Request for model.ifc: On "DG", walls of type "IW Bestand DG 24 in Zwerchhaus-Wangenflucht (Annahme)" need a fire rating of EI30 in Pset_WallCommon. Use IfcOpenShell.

First a look at what the model holds.

```python
import ifcopenshell
import ifcopenshell.util.element

model = ifcopenshell.open("model.ifc")
print(model.schema)
storey = next(s for s in model.by_type("IfcBuildingStorey") if s.Name == "DG")
walls = [e for e in ifcopenshell.util.element.get_decomposition(storey) if e.is_a("IfcWall")]
seen = {}
for e in walls:
    element_type = ifcopenshell.util.element.get_type(e)
    key = (element_type.Name if element_type != e and element_type else None, ifcopenshell.util.element.get_pset(e, "Pset_WallCommon", "FireRating"))
    seen[key] = seen.get(key, 0) + 1
for (name, value), count in sorted(seen.items(), key=str):
    print(count, "x", name, "|", value)
```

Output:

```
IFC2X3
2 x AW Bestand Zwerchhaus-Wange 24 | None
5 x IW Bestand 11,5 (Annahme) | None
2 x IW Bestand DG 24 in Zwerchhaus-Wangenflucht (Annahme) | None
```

```python
import ifcopenshell
import ifcopenshell.api.pset
import ifcopenshell.util.element

model = ifcopenshell.open("model.ifc")

storey = next(s for s in model.by_type("IfcBuildingStorey") if s.Name == "DG")
walls = [e for e in ifcopenshell.util.element.get_decomposition(storey) if e.is_a("IfcWall")]

count = 0
for e in walls:
    element_type = ifcopenshell.util.element.get_type(e)
    if element_type in (None, e) or element_type.Name != "IW Bestand DG 24 in Zwerchhaus-Wangenflucht (Annahme)":
        continue
    # add_pset returns the element's existing set when there is one.
    pset = ifcopenshell.api.pset.add_pset(model, product=e, name="Pset_WallCommon")
    ifcopenshell.api.pset.edit_pset(model, pset=pset, properties={"FireRating": "EI30"})
    count += 1

print(count, "walls updated")

model.write("model_v2.ifc")
```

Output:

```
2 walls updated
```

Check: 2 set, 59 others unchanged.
